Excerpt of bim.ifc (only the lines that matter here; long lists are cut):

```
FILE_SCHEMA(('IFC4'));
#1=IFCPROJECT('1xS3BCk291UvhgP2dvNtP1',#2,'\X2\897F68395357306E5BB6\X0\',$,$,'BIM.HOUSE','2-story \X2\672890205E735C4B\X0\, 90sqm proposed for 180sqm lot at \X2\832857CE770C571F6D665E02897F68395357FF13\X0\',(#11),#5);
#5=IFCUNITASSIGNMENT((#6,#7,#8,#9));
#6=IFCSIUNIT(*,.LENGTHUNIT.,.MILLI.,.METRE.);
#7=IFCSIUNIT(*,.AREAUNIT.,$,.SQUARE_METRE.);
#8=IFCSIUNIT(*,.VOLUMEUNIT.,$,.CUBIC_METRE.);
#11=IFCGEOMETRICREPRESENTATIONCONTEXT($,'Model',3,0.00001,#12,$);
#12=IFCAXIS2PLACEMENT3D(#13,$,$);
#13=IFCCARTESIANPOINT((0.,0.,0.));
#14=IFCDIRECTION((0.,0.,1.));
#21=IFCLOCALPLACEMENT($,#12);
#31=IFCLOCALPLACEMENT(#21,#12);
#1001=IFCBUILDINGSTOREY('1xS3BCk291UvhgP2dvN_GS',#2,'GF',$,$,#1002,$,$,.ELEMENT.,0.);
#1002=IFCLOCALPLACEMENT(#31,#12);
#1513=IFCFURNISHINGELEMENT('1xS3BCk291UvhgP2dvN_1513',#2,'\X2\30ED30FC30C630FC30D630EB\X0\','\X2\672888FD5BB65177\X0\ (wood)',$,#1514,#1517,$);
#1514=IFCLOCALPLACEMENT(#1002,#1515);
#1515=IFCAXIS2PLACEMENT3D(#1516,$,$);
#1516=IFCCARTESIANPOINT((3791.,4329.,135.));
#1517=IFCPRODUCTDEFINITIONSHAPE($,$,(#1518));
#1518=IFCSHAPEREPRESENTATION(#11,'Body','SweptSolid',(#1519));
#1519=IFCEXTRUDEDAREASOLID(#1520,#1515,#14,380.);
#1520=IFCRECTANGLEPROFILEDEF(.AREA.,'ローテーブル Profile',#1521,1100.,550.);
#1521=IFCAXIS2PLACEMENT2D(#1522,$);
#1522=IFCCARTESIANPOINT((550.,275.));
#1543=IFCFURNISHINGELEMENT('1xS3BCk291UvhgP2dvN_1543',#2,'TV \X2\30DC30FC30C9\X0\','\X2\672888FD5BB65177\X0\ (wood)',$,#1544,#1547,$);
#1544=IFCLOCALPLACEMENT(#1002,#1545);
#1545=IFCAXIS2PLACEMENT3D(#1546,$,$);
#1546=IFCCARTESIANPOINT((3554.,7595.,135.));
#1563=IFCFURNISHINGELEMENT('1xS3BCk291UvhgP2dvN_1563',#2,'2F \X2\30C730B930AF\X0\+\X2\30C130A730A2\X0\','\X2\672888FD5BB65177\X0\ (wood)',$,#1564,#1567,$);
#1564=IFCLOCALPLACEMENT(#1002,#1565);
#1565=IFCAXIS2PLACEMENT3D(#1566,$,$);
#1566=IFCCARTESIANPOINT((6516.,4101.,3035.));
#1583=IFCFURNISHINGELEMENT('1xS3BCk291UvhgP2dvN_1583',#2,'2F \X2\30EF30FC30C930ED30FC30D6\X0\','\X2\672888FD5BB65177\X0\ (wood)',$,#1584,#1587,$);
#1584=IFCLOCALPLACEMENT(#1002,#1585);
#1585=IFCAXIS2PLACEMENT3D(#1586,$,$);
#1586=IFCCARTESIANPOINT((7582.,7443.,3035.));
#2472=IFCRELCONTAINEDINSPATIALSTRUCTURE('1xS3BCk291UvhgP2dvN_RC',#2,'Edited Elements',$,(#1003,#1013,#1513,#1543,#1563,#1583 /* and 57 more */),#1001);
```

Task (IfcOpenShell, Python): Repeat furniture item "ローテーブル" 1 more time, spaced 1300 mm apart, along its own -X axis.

```python
import ifcopenshell
import ifcopenshell.api.geometry
import ifcopenshell.api.root
import ifcopenshell.util.element
import ifcopenshell.util.placement

model = ifcopenshell.open("bim.ifc")


def reuse_history(source, copy):
    """copy_class also copies each property set's owner history, people and application; keep the originals."""
    for rel in copy.IsDefinedBy:
        if rel.is_a("IfcRelDefinesByProperties") and (history := rel.RelatingPropertyDefinition.OwnerHistory):
            rel.RelatingPropertyDefinition.OwnerHistory = source.OwnerHistory
            ifcopenshell.util.element.remove_deep2(model, history)


source = model.by_id(1513)
base = ifcopenshell.util.placement.get_local_placement(source.ObjectPlacement)
step = -base[:3, 0] * 1300.0

for i in range(1, 2):
    copy = ifcopenshell.api.root.copy_class(model, product=source)
    copy.Representation = ifcopenshell.util.element.copy_deep(
        model, source.Representation, exclude=["IfcGeometricRepresentationContext", "IfcRepresentationMap"]
    )
    reuse_history(source, copy)
    matrix = base.copy()
    matrix[:3, 3] += i * step
    print("added at", matrix[:3, 3].round(3) + 0.0)
    ifcopenshell.api.geometry.edit_object_placement(model, product=copy, matrix=matrix, is_si=False)

model.write("bim-out.ifc")
```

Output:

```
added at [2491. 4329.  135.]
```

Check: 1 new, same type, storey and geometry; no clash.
